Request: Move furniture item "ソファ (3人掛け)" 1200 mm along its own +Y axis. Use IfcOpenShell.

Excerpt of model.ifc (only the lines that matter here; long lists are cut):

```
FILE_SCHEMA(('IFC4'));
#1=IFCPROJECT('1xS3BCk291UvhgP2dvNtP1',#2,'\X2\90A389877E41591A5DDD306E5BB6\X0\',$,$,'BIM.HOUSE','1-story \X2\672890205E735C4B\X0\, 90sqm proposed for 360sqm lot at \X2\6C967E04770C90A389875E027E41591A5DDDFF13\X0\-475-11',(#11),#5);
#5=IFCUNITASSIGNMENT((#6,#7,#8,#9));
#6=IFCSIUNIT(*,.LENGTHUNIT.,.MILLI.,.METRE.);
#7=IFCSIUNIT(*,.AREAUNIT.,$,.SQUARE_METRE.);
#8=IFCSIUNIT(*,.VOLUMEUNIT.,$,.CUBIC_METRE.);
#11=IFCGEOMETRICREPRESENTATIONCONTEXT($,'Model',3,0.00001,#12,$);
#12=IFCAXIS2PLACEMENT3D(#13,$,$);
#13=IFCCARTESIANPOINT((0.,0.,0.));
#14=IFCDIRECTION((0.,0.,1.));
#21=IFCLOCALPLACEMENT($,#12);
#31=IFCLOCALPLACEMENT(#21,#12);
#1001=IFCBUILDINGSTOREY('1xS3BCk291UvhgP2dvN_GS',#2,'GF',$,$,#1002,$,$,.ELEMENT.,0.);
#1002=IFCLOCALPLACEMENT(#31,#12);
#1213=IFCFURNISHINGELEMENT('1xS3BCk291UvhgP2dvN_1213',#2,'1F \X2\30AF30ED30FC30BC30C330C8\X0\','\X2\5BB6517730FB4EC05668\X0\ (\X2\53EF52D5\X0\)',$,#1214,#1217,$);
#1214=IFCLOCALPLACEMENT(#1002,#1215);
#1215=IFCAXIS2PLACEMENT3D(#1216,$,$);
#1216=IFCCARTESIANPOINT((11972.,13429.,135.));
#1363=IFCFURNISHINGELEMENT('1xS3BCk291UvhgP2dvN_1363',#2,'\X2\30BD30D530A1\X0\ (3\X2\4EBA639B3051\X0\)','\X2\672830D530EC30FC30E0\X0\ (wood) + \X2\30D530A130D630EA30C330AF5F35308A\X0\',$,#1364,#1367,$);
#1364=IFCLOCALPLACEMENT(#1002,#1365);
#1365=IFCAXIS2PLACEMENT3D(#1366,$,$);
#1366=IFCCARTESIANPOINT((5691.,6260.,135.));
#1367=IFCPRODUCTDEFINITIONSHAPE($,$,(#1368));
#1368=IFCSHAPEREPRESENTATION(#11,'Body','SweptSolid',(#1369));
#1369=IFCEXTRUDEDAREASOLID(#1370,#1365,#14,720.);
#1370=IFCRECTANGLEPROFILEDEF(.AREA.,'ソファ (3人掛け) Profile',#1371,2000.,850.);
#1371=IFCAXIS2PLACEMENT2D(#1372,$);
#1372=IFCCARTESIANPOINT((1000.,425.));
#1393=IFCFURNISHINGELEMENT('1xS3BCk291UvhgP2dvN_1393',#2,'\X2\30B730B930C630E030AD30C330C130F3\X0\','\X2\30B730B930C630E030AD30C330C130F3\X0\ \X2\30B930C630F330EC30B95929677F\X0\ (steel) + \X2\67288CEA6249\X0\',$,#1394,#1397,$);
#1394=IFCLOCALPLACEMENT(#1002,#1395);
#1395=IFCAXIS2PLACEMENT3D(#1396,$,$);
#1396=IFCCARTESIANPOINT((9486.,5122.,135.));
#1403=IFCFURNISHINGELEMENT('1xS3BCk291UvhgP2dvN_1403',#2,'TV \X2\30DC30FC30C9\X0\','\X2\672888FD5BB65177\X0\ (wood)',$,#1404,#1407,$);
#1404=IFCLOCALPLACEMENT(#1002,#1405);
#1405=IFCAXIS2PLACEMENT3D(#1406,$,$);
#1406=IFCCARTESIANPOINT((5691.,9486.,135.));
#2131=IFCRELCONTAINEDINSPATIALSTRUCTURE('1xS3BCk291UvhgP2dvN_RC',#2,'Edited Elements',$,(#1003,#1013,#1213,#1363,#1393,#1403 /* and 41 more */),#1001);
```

```python
import ifcopenshell
import ifcopenshell.api.geometry
import ifcopenshell.util.placement

model = ifcopenshell.open("model.ifc")

item = model.by_id(1363)
matrix = ifcopenshell.util.placement.get_local_placement(item.ObjectPlacement)
matrix[:3, 3] += matrix[:3, 1] * 1200.0
ifcopenshell.api.geometry.edit_object_placement(model, product=item, matrix=matrix, is_si=False)

print(ifcopenshell.util.placement.get_local_placement(item.ObjectPlacement).round(3) + 0.0)

model.write("model_edited.ifc")
```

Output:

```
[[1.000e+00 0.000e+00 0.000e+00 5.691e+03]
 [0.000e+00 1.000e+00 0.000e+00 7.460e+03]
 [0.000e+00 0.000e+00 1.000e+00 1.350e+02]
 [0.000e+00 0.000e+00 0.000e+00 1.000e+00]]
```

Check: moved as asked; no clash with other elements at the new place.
